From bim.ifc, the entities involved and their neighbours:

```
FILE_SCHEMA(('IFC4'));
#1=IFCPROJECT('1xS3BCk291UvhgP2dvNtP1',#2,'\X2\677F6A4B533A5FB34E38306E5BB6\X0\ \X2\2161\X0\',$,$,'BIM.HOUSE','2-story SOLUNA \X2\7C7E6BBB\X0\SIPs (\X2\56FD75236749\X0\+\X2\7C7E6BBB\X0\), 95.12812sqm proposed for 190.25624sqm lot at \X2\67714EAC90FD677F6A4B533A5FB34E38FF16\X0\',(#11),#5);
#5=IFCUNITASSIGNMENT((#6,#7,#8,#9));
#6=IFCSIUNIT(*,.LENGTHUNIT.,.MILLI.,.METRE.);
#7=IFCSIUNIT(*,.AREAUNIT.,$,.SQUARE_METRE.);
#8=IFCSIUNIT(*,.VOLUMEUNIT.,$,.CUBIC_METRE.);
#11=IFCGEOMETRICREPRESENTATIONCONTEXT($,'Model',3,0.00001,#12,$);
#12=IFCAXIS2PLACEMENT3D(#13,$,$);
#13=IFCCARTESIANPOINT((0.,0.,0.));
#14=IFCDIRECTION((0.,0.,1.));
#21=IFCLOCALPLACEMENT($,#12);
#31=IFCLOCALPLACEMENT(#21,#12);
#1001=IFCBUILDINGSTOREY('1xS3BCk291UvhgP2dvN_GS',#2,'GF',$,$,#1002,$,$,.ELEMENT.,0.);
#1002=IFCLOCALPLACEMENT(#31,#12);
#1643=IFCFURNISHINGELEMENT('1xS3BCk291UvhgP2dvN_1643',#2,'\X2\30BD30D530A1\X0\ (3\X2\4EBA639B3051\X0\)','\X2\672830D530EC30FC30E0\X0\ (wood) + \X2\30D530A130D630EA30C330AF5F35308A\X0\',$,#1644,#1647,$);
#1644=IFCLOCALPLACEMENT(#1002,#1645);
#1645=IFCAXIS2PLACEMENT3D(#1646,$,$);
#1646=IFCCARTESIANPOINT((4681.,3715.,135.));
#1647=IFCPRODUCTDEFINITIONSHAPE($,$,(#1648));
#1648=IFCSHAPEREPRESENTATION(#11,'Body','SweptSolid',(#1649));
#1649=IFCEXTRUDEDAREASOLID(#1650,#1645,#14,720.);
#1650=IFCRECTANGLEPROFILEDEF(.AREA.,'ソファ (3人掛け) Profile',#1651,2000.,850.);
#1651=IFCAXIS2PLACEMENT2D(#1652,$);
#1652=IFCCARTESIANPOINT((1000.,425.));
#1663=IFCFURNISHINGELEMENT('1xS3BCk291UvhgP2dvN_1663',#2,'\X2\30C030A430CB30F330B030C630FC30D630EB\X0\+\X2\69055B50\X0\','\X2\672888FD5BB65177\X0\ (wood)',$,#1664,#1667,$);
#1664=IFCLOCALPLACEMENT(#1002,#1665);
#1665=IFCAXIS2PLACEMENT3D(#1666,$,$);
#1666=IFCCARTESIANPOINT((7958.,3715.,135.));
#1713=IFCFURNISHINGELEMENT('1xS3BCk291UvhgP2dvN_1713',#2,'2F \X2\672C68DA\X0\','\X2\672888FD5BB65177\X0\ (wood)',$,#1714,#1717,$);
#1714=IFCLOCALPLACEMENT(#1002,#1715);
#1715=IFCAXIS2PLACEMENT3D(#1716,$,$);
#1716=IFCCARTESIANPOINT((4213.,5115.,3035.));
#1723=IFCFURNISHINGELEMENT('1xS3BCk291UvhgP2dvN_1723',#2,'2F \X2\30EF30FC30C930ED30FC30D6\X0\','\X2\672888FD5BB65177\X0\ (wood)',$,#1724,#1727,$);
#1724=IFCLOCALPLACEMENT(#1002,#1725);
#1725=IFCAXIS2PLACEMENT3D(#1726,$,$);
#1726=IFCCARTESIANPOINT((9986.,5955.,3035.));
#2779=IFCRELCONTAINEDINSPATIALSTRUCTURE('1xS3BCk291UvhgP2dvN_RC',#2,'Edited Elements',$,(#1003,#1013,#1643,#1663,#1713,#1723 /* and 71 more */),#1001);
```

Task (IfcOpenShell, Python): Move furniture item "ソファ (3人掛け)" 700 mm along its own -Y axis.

```python
import ifcopenshell
import ifcopenshell.api.geometry
import ifcopenshell.util.placement
import ifcopenshell.util.unit

model = ifcopenshell.open("bim.ifc")
unit_scale = ifcopenshell.util.unit.calculate_unit_scale(model)

item = model.by_guid("1xS3BCk291UvhgP2dvN_1643")
matrix = ifcopenshell.util.placement.get_local_placement(item.ObjectPlacement)
matrix[:3, 3] -= matrix[:3, 1] * 0.7 / unit_scale
ifcopenshell.api.geometry.edit_object_placement(model, product=item, matrix=matrix, is_si=False)

print(ifcopenshell.util.placement.get_local_placement(item.ObjectPlacement).round(3) + 0.0)

model.write("bim-out.ifc")
```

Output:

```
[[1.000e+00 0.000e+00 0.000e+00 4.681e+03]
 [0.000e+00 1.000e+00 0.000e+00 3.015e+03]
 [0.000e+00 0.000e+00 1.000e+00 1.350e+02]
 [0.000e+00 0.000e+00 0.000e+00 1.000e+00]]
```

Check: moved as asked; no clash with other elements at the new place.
